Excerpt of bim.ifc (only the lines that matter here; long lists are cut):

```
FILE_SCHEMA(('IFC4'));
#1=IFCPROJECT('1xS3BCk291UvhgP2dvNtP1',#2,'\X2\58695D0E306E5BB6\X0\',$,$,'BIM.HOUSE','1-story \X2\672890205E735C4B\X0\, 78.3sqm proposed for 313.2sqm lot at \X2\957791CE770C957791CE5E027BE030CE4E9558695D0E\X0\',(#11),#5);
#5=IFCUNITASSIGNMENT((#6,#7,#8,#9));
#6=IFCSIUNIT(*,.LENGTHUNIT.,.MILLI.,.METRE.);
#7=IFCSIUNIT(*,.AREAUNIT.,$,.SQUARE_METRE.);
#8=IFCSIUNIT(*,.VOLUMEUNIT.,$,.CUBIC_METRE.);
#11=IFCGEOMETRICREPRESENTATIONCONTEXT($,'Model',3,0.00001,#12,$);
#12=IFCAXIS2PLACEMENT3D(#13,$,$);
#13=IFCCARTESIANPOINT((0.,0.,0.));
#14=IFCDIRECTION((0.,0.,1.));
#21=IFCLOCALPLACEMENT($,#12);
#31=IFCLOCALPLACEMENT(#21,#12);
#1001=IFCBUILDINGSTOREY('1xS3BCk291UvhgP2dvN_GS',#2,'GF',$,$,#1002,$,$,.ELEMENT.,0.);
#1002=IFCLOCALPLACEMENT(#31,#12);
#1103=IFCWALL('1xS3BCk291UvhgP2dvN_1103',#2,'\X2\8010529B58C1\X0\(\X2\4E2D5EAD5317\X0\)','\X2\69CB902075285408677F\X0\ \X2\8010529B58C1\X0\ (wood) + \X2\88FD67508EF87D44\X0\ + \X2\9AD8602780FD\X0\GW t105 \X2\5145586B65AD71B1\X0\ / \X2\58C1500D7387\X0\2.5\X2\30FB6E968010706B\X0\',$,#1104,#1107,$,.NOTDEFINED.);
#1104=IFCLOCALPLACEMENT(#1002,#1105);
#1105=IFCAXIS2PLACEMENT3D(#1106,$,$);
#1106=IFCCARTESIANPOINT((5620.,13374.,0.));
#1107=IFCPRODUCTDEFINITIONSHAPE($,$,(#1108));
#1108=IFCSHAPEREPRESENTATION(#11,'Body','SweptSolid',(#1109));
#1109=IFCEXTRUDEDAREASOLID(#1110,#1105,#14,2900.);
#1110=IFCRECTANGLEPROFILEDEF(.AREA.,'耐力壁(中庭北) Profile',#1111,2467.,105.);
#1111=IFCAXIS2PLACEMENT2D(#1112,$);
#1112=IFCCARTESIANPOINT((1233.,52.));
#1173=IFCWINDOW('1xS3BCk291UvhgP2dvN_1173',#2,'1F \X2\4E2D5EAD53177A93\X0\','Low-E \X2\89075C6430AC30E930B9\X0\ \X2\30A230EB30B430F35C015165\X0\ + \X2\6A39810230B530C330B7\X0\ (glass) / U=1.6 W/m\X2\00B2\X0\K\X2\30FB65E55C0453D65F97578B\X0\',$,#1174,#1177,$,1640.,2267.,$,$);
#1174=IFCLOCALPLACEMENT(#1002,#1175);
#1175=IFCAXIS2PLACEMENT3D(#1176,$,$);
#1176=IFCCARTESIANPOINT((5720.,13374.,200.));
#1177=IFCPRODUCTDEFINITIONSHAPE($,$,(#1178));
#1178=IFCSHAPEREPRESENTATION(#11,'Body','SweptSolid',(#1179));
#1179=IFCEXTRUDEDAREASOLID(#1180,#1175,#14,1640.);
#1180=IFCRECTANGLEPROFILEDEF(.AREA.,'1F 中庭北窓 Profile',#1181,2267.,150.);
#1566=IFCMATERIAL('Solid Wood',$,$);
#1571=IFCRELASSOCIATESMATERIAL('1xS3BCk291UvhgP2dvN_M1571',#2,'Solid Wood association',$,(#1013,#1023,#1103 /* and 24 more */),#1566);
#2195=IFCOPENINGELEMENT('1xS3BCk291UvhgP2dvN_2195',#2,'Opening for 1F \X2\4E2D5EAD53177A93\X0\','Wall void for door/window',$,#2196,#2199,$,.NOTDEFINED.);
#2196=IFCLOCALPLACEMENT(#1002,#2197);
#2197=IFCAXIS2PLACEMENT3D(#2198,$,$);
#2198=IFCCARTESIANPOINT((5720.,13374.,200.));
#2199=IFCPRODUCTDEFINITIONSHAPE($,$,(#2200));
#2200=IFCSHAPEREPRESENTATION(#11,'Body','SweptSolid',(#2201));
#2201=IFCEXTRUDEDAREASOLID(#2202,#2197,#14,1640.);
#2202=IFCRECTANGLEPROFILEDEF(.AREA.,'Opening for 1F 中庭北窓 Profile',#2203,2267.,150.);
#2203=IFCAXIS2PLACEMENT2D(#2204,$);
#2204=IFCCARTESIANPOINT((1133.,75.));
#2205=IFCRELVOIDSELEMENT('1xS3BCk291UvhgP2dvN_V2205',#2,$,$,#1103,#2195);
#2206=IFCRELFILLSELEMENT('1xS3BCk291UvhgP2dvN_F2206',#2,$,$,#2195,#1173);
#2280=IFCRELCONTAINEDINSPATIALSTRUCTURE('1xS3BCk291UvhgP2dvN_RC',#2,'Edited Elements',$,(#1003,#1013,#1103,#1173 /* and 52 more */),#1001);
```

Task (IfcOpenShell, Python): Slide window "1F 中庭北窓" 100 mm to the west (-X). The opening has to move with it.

```python
import ifcopenshell
import ifcopenshell.api.geometry
import ifcopenshell.util.placement

model = ifcopenshell.open("bim.ifc")

window = model.by_guid("1xS3BCk291UvhgP2dvN_1173")
opening = window.FillsVoids[0].RelatingOpeningElement
wall = opening.VoidsElements[0].RelatingBuildingElement

wall_matrix = ifcopenshell.util.placement.get_local_placement(wall.ObjectPlacement)
shift = wall_matrix[:3, 0] * -100.0
before = ifcopenshell.util.placement.get_local_placement(window.ObjectPlacement)[:3, 3].copy()

# The window is not placed relative to its opening, so move both.
for product in (opening, window):
    matrix = ifcopenshell.util.placement.get_local_placement(product.ObjectPlacement)
    matrix[:3, 3] += shift
    ifcopenshell.api.geometry.edit_object_placement(model, product=product, matrix=matrix, is_si=False)

after = ifcopenshell.util.placement.get_local_placement(window.ObjectPlacement)[:3, 3]
print("window moved by", (after - before).round(3) + 0.0)

model.write("bim_v2.ifc")
```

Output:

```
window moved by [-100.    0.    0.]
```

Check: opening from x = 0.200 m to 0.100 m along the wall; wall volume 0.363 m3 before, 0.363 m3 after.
